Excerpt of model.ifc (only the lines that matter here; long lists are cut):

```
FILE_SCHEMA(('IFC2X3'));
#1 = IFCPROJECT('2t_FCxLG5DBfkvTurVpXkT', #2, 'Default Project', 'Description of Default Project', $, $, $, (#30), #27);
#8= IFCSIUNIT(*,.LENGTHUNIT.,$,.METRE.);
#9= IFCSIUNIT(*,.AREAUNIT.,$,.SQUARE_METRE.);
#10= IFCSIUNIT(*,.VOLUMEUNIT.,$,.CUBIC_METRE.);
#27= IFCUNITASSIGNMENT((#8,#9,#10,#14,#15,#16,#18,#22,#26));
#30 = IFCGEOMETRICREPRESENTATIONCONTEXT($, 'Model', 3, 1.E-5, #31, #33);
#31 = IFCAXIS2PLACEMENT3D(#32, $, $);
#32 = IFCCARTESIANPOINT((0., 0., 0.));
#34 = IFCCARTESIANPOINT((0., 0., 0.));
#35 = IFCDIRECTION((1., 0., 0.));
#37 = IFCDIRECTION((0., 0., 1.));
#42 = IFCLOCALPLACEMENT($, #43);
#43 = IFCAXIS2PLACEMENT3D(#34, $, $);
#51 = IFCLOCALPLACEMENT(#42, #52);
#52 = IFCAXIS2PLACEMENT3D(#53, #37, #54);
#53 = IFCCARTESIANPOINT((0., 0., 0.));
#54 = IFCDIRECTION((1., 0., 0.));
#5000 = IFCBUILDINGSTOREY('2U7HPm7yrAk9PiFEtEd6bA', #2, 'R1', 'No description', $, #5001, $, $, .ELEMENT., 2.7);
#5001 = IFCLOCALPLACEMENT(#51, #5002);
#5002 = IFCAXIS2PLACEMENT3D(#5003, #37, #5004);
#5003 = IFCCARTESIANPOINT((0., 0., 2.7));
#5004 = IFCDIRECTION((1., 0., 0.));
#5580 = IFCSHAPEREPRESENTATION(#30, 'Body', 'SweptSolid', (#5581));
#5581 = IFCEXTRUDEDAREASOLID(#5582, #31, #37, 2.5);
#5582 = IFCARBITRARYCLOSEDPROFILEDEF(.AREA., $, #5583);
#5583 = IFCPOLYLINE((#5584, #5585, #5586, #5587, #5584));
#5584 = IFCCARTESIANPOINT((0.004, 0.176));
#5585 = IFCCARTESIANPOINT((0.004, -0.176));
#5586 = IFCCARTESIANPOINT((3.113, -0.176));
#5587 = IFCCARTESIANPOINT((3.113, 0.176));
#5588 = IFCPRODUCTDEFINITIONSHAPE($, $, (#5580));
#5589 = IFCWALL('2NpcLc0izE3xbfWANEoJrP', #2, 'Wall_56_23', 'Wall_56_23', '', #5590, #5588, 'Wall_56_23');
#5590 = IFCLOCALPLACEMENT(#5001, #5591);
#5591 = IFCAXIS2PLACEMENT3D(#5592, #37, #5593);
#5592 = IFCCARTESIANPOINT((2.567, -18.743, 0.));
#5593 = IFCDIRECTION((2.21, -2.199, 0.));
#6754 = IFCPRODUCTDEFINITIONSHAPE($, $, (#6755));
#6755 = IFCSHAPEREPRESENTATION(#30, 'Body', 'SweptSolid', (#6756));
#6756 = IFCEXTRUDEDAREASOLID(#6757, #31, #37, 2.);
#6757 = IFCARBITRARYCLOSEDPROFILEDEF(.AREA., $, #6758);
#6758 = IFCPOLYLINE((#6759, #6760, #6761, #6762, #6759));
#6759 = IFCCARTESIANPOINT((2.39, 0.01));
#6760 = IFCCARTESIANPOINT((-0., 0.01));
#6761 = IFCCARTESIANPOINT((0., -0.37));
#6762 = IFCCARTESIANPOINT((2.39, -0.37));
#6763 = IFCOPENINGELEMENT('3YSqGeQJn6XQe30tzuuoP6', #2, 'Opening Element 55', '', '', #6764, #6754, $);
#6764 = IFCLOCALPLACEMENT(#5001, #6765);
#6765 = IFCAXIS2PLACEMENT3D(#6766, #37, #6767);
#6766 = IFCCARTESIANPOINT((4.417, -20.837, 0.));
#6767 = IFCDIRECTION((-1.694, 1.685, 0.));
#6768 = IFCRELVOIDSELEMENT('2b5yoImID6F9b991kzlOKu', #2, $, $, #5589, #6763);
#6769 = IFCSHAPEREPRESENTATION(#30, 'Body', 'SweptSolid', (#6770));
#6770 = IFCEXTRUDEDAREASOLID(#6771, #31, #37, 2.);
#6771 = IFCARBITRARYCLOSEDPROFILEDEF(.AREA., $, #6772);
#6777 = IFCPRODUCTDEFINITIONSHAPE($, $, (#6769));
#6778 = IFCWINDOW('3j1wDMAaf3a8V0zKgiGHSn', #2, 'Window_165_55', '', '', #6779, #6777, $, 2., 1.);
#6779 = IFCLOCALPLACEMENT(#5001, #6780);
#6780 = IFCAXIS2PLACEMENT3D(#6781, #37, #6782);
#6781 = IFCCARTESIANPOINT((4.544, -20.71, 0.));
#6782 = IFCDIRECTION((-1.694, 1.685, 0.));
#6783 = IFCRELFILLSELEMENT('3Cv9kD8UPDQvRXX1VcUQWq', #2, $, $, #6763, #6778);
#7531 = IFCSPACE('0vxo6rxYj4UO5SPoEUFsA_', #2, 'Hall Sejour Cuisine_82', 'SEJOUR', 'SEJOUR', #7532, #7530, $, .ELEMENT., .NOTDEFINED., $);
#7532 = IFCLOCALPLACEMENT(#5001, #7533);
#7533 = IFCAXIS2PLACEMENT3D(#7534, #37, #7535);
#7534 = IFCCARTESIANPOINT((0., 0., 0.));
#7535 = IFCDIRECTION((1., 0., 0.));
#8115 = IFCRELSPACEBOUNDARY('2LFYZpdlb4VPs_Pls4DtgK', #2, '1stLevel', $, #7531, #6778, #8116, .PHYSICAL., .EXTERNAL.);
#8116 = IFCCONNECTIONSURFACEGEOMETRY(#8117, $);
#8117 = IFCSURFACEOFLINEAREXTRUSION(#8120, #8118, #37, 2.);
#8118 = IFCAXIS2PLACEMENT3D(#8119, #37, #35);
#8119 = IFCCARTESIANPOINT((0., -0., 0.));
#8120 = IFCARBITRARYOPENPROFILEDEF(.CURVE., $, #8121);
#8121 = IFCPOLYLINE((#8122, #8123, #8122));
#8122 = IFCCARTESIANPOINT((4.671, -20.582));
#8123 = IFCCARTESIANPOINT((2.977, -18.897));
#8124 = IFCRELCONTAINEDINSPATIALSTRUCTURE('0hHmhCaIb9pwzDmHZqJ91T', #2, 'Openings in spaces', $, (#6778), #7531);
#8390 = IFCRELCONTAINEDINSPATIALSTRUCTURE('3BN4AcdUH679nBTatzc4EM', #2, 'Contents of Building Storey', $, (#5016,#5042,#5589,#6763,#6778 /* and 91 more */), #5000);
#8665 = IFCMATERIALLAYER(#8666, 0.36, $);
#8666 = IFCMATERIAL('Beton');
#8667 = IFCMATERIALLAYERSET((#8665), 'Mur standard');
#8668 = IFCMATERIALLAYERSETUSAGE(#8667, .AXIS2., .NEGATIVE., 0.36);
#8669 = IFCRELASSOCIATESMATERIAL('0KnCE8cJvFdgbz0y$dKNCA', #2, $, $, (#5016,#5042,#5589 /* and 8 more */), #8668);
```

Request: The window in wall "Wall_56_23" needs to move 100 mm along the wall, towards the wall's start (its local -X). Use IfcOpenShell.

```python
import numpy as np
import ifcopenshell
import ifcopenshell.api.geometry
import ifcopenshell.util.placement
import ifcopenshell.util.unit

model = ifcopenshell.open("model.ifc")
unit_scale = ifcopenshell.util.unit.calculate_unit_scale(model)

window = model.by_guid("3j1wDMAaf3a8V0zKgiGHSn")
opening = window.FillsVoids[0].RelatingOpeningElement
wall = opening.VoidsElements[0].RelatingBuildingElement

wall_matrix = ifcopenshell.util.placement.get_local_placement(wall.ObjectPlacement)
shift = wall_matrix[:3, 0] * -0.1 / unit_scale
before = ifcopenshell.util.placement.get_local_placement(window.ObjectPlacement)[:3, 3].copy()

# The window is not placed relative to its opening, so move both.
for product in (opening, window):
    matrix = ifcopenshell.util.placement.get_local_placement(product.ObjectPlacement)
    matrix[:3, 3] += shift
    ifcopenshell.api.geometry.edit_object_placement(model, product=product, matrix=matrix, is_si=False)

# Space boundary surfaces are stored in each space's coordinates; move them too.
for rel in window.ProvidesBoundaries:
    if not rel.ConnectionGeometry:
        continue
    surface = rel.ConnectionGeometry.SurfaceOnRelatingElement
    space_matrix = ifcopenshell.util.placement.get_local_placement(rel.RelatingSpace.ObjectPlacement)
    point = np.array(surface.Position.Location.Coordinates) + space_matrix[:3, :3].T @ shift
    surface.Position = model.createIfcAxis2Placement3D(
        model.createIfcCartesianPoint(point.tolist()), surface.Position.Axis, surface.Position.RefDirection
    )

after = ifcopenshell.util.placement.get_local_placement(window.ObjectPlacement)[:3, 3]
print("window moved by", (after - before).round(3) + 0.0)

model.write("model-out.ifc")
```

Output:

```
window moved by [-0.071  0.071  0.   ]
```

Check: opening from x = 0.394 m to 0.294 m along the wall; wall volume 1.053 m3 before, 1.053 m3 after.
